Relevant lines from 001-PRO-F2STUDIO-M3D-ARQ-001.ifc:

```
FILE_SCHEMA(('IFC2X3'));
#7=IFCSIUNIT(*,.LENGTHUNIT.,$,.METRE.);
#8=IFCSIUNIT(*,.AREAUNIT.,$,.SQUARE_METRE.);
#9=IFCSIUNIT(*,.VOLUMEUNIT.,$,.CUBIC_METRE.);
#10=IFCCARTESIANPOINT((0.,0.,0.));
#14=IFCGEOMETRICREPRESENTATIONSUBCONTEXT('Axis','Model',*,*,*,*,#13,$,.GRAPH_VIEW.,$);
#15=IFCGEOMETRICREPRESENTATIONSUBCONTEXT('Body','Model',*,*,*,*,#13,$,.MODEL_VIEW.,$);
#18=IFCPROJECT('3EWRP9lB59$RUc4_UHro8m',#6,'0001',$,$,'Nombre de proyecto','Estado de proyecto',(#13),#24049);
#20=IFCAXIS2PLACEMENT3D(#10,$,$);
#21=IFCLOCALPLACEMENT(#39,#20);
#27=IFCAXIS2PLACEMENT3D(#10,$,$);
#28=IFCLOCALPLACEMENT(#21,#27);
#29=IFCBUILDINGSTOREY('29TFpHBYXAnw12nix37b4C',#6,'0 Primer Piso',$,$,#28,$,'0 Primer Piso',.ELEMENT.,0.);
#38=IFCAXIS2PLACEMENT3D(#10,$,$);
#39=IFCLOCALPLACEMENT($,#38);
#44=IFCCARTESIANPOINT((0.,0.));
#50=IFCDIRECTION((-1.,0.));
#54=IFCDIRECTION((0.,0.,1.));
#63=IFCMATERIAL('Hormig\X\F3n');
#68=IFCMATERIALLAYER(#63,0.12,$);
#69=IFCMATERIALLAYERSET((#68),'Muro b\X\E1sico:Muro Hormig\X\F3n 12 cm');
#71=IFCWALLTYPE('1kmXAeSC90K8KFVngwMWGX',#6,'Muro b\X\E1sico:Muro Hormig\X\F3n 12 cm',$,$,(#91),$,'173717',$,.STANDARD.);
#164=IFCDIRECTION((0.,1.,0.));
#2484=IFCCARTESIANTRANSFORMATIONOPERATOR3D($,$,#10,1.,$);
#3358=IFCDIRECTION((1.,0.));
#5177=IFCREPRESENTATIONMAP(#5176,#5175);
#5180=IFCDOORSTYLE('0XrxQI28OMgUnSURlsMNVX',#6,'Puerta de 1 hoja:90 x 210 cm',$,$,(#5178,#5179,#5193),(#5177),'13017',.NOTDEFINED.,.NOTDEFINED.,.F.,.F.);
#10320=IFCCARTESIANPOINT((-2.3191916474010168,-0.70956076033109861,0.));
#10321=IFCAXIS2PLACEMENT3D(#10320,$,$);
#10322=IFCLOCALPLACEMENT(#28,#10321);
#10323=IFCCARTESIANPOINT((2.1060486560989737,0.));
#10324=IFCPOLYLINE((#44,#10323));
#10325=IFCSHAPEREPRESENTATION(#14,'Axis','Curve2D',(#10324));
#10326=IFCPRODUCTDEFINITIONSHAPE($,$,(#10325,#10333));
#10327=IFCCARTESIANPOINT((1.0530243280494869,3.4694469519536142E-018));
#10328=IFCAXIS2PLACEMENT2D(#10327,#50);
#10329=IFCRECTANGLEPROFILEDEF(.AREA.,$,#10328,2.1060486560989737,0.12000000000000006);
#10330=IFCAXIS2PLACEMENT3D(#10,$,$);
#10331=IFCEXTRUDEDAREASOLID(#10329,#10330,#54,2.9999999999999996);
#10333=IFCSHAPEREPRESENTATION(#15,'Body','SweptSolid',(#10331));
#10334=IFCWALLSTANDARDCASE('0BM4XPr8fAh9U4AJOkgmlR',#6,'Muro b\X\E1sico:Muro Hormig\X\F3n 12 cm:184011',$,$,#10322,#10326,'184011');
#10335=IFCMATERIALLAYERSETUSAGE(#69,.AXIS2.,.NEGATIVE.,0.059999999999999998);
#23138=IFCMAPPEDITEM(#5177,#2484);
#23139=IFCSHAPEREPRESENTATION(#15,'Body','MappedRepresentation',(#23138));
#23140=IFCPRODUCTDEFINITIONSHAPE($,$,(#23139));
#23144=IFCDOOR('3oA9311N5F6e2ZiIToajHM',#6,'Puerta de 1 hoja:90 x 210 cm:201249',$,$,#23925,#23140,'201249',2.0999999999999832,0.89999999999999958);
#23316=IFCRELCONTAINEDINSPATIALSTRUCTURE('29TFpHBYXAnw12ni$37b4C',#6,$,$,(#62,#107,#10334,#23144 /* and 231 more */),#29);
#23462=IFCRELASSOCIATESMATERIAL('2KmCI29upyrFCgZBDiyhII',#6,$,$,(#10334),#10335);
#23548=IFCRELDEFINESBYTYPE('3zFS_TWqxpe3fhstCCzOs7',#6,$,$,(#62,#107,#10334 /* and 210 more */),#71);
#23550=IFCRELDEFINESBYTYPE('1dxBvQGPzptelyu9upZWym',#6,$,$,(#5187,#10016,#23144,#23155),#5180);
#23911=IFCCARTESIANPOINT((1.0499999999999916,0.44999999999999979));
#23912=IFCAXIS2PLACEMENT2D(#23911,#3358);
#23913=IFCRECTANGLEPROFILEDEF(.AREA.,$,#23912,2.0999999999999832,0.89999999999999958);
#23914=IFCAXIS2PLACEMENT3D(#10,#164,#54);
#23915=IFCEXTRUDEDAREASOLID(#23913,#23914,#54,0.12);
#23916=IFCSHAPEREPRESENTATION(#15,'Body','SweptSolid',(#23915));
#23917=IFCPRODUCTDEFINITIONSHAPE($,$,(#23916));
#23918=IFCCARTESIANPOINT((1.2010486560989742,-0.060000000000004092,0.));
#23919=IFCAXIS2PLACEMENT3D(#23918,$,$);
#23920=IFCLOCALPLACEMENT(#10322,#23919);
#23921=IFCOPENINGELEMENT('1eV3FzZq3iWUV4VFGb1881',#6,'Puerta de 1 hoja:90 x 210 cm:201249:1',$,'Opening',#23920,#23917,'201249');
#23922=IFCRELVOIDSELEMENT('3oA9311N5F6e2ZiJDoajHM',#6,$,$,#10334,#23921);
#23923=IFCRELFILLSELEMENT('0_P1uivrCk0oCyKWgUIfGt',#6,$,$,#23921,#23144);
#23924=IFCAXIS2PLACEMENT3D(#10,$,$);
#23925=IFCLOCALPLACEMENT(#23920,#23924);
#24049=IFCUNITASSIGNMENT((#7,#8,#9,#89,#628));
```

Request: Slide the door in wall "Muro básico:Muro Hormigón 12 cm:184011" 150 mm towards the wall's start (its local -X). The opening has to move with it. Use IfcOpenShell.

```python
import ifcopenshell
import ifcopenshell.api.geometry
import ifcopenshell.util.placement
import ifcopenshell.util.unit

model = ifcopenshell.open("001-PRO-F2STUDIO-M3D-ARQ-001.ifc")
unit_scale = ifcopenshell.util.unit.calculate_unit_scale(model)

door = model.by_id(23144)
opening = door.FillsVoids[0].RelatingOpeningElement
wall = opening.VoidsElements[0].RelatingBuildingElement

wall_matrix = ifcopenshell.util.placement.get_local_placement(wall.ObjectPlacement)
shift = wall_matrix[:3, 0] * -0.15 / unit_scale
before = ifcopenshell.util.placement.get_local_placement(door.ObjectPlacement)[:3, 3].copy()

# The door is placed relative to its opening, so it follows when the opening moves.
matrix = ifcopenshell.util.placement.get_local_placement(opening.ObjectPlacement)
matrix[:3, 3] += shift
ifcopenshell.api.geometry.edit_object_placement(
    model, product=opening, matrix=matrix, is_si=False, should_transform_children=True
)

after = ifcopenshell.util.placement.get_local_placement(door.ObjectPlacement)[:3, 3]
print("door moved by", (after - before).round(3) + 0.0)

model.write("001-PRO-F2STUDIO-M3D-ARQ-001_rev.ifc")
```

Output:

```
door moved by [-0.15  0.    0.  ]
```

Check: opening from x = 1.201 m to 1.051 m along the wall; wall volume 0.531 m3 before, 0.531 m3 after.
